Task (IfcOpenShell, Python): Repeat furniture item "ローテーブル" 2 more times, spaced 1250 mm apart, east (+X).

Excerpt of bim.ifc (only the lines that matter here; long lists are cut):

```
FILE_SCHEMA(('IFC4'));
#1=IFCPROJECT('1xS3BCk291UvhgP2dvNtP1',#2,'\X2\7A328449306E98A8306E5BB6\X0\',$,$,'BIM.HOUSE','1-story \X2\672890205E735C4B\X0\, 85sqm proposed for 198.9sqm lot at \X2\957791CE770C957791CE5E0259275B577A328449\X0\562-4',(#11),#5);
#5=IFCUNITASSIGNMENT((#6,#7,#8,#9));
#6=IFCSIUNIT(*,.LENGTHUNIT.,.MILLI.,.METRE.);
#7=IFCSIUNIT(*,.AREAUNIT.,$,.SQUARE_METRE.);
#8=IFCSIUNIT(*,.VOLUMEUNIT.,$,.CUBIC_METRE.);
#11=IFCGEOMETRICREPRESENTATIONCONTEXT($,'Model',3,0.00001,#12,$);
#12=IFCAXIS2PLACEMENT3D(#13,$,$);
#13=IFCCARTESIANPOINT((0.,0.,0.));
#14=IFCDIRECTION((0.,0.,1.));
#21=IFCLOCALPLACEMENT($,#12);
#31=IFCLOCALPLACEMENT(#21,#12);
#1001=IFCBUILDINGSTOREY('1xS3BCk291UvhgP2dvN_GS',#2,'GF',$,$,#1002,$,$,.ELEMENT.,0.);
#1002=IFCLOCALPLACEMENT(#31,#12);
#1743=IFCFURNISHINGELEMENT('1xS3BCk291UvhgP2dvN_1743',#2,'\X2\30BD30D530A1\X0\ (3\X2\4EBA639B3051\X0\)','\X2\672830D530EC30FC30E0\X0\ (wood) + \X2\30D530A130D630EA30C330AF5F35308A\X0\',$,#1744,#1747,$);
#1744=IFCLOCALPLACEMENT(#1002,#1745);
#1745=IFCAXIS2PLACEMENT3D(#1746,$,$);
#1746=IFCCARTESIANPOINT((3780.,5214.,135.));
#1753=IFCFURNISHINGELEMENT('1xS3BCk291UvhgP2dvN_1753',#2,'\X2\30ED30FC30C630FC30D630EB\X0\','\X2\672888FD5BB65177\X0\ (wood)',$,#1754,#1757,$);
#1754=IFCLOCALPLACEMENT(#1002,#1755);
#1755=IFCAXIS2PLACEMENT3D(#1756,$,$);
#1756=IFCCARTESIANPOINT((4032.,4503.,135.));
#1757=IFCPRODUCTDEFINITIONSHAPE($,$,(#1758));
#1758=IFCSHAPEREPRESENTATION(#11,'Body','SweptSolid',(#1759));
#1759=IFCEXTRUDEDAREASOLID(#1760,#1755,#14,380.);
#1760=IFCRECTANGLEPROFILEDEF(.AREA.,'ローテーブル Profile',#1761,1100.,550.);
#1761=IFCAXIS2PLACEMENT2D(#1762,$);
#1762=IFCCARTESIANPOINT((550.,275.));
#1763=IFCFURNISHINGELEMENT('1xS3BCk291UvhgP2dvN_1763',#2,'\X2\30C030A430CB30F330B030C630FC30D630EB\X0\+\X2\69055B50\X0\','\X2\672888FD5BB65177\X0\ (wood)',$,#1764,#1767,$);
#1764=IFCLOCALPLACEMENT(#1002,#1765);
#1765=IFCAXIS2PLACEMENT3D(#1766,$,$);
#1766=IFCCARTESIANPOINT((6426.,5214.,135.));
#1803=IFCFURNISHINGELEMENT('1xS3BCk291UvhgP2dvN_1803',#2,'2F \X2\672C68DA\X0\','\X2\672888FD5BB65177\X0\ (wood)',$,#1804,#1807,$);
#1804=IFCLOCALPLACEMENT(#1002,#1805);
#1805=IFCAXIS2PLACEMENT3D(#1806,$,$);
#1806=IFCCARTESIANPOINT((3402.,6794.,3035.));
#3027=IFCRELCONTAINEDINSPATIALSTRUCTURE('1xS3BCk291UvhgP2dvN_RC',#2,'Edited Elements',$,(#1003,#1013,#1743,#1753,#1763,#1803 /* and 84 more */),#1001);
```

```python
import numpy as np
import ifcopenshell
import ifcopenshell.api.geometry
import ifcopenshell.api.root
import ifcopenshell.util.element
import ifcopenshell.util.placement
import ifcopenshell.util.unit

model = ifcopenshell.open("bim.ifc")
unit_scale = ifcopenshell.util.unit.calculate_unit_scale(model)


def reuse_history(source, copy):
    """copy_class also copies each property set's owner history, people and application; keep the originals."""
    for rel in copy.IsDefinedBy:
        if rel.is_a("IfcRelDefinesByProperties") and (history := rel.RelatingPropertyDefinition.OwnerHistory):
            rel.RelatingPropertyDefinition.OwnerHistory = source.OwnerHistory
            ifcopenshell.util.element.remove_deep2(model, history)


source = model.by_guid("1xS3BCk291UvhgP2dvN_1753")
base = ifcopenshell.util.placement.get_local_placement(source.ObjectPlacement)
step = np.array([1.0, 0.0, 0.0]) * 1.25 / unit_scale

for i in range(1, 3):
    copy = ifcopenshell.api.root.copy_class(model, product=source)
    copy.Representation = ifcopenshell.util.element.copy_deep(
        model, source.Representation, exclude=["IfcGeometricRepresentationContext", "IfcRepresentationMap"]
    )
    reuse_history(source, copy)
    matrix = base.copy()
    matrix[:3, 3] += i * step
    print("added at", matrix[:3, 3].round(3) + 0.0)
    ifcopenshell.api.geometry.edit_object_placement(model, product=copy, matrix=matrix, is_si=False)

model.write("bim_edited.ifc")
```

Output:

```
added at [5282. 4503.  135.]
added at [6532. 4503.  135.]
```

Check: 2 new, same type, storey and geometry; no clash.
